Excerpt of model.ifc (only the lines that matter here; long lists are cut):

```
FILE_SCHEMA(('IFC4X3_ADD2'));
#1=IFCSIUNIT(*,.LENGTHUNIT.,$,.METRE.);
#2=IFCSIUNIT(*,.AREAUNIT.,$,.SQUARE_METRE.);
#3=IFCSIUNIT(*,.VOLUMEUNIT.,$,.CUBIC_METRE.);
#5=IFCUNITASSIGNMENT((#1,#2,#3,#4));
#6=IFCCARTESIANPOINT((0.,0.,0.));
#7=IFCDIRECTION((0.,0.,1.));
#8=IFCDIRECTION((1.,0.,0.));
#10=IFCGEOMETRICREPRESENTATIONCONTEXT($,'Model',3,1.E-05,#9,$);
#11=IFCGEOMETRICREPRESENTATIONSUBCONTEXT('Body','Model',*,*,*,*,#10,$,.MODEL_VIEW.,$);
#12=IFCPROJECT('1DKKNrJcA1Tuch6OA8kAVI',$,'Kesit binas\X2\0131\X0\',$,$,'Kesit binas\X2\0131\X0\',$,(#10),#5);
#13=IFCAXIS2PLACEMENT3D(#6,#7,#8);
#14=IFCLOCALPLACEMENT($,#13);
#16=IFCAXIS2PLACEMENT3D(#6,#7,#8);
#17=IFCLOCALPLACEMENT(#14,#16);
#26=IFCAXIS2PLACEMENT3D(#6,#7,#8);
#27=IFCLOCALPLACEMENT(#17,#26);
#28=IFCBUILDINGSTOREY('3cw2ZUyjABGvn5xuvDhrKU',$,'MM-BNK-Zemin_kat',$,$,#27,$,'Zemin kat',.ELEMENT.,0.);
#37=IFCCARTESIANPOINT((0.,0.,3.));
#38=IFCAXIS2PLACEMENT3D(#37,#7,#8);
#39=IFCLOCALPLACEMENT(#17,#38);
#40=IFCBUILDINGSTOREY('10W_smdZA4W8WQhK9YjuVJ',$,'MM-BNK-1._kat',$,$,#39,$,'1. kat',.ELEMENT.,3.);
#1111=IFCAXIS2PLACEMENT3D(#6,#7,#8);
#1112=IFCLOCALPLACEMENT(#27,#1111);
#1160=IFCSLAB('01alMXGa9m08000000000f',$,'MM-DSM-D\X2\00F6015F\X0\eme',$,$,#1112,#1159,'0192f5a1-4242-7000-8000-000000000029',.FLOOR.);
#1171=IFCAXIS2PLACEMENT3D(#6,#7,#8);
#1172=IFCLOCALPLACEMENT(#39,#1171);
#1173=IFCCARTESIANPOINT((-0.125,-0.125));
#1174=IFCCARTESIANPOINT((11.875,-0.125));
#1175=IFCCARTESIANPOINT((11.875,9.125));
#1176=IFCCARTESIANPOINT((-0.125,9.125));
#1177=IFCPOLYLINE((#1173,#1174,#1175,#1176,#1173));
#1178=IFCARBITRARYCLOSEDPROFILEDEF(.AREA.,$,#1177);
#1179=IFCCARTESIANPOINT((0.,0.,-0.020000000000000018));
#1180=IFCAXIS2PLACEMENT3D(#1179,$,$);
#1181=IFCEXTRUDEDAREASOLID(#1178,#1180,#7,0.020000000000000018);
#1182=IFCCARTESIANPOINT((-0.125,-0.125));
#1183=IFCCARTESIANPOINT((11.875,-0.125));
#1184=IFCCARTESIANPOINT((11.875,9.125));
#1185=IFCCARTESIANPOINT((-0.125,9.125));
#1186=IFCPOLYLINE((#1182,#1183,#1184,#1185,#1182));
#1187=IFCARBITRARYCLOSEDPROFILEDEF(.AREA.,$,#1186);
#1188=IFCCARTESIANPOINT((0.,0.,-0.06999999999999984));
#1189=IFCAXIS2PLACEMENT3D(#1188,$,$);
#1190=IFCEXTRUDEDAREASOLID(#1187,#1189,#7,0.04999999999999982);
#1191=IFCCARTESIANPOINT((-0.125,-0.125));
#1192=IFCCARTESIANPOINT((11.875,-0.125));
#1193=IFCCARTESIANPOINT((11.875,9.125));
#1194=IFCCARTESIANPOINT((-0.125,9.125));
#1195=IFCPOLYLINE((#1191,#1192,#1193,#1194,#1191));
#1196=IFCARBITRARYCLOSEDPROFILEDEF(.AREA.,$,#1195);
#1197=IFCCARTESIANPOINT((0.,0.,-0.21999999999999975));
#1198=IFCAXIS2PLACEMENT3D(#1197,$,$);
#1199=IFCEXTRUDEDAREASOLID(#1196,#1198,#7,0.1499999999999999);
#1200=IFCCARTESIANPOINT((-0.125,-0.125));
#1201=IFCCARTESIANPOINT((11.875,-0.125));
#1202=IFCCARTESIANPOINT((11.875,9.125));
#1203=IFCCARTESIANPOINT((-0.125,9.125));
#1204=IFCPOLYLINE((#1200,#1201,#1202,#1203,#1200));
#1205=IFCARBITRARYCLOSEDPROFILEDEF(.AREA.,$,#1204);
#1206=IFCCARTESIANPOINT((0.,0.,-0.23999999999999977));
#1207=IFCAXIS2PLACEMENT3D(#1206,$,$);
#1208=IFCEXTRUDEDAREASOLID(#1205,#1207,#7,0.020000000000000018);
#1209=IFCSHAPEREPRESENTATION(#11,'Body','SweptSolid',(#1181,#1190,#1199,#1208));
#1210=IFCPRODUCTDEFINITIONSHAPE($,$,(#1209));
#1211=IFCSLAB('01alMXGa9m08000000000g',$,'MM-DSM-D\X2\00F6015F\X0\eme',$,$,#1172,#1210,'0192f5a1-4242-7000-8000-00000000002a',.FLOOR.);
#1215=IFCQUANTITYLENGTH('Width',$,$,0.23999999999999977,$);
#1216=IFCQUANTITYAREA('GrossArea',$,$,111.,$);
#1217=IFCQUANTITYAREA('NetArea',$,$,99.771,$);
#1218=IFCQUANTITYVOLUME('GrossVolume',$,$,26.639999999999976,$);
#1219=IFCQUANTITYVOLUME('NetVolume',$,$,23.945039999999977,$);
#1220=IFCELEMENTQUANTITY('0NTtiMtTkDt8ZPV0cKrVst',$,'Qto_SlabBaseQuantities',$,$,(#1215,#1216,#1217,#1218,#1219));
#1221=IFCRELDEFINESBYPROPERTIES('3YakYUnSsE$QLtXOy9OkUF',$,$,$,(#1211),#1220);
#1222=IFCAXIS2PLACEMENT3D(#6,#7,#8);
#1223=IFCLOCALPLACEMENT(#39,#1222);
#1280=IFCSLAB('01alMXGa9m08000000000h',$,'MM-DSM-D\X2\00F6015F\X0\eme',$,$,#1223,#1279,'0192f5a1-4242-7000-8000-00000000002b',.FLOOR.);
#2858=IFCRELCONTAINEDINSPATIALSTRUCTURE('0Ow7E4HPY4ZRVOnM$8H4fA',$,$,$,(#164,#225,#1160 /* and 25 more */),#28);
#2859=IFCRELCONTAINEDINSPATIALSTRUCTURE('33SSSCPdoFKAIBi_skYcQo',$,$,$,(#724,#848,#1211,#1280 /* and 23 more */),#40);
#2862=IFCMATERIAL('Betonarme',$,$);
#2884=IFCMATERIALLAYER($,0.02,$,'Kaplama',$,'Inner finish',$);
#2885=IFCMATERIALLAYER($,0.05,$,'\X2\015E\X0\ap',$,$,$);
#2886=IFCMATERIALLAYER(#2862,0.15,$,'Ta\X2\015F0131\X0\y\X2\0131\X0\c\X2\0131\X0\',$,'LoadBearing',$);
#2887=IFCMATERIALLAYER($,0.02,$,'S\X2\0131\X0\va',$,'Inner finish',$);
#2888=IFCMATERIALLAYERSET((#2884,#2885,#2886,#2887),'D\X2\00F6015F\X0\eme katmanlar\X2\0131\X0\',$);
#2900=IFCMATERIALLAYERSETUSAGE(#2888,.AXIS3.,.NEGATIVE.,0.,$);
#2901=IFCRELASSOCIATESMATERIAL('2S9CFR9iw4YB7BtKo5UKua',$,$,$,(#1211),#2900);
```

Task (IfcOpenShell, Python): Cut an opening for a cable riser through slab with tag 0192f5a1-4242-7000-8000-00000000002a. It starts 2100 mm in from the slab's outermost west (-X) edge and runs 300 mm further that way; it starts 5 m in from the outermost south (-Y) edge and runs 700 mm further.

```python
import numpy as np
import ifcopenshell
import ifcopenshell.api.feature
import ifcopenshell.api.geometry
import ifcopenshell.api.pset
import ifcopenshell.api.root
import ifcopenshell.geom
import ifcopenshell.util.element
import ifcopenshell.util.placement
import ifcopenshell.util.representation
import ifcopenshell.util.shape
import ifcopenshell.util.unit

model = ifcopenshell.open("model.ifc")
unit_scale = ifcopenshell.util.unit.calculate_unit_scale(model)
area_scale = ifcopenshell.util.unit.calculate_unit_scale(model, "AREAUNIT")
volume_scale = ifcopenshell.util.unit.calculate_unit_scale(model, "VOLUMEUNIT")
settings = ifcopenshell.geom.settings()


def volume(element):
    """Net volume in cubic metres, openings subtracted."""
    shape = ifcopenshell.geom.create_shape(settings, element)
    return ifcopenshell.util.shape.get_volume(shape.geometry)


slab = model.by_id(1211)
before = volume(slab)

# Extent in the slab's own axes, in metres. The edges named are its -X and -Y sides.
slab_shape = ifcopenshell.geom.create_shape(settings, slab)
vertices = ifcopenshell.util.shape.get_vertices(slab_shape.geometry)
x_min, y_min, bottom = vertices.min(axis=0)
top = vertices[:, 2].max()

opening = ifcopenshell.api.root.create_entity(model, ifc_class="IfcOpeningElement", name="Cable riser opening", predefined_type="OPENING")
context = ifcopenshell.util.representation.get_context(model, "Model", "Body", "MODEL_VIEW")
width, depth = 0.3, 0.7
outline = [(0.0, 0.0), (width, 0.0), (width, depth), (0.0, depth), (0.0, 0.0)]
# Overshoot both faces by 50 mm so the cut is clean.
shape = ifcopenshell.api.geometry.add_slab_representation(
    model, context=context, depth=top - bottom + 0.1, polyline=outline
)
ifcopenshell.api.geometry.assign_representation(model, product=opening, representation=shape)

matrix = ifcopenshell.util.placement.get_local_placement(slab.ObjectPlacement)
matrix[:, 3] = matrix @ np.append(np.array([x_min + 2.1, y_min + 5, bottom - 0.05]) / unit_scale, 1.0)
ifcopenshell.api.geometry.edit_object_placement(model, product=opening, matrix=matrix, is_si=False)
ifcopenshell.api.feature.add_feature(model, feature=opening, element=slab)

after = volume(slab)

# Update the slab's stored quantities.
qto = model.by_id(ifcopenshell.util.element.get_pset(slab, "Qto_SlabBaseQuantities", should_inherit=False)["id"])
ifcopenshell.api.pset.edit_qto(model, qto=qto, properties={
    "NetArea": after / (top - bottom) / area_scale,
    "NetVolume": after / volume_scale,
})

print(f"slab volume {before:.3f} -> {after:.3f} m3")

model.write("model-out.ifc")
```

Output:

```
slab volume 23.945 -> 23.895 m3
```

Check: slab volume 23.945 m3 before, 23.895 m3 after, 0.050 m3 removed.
